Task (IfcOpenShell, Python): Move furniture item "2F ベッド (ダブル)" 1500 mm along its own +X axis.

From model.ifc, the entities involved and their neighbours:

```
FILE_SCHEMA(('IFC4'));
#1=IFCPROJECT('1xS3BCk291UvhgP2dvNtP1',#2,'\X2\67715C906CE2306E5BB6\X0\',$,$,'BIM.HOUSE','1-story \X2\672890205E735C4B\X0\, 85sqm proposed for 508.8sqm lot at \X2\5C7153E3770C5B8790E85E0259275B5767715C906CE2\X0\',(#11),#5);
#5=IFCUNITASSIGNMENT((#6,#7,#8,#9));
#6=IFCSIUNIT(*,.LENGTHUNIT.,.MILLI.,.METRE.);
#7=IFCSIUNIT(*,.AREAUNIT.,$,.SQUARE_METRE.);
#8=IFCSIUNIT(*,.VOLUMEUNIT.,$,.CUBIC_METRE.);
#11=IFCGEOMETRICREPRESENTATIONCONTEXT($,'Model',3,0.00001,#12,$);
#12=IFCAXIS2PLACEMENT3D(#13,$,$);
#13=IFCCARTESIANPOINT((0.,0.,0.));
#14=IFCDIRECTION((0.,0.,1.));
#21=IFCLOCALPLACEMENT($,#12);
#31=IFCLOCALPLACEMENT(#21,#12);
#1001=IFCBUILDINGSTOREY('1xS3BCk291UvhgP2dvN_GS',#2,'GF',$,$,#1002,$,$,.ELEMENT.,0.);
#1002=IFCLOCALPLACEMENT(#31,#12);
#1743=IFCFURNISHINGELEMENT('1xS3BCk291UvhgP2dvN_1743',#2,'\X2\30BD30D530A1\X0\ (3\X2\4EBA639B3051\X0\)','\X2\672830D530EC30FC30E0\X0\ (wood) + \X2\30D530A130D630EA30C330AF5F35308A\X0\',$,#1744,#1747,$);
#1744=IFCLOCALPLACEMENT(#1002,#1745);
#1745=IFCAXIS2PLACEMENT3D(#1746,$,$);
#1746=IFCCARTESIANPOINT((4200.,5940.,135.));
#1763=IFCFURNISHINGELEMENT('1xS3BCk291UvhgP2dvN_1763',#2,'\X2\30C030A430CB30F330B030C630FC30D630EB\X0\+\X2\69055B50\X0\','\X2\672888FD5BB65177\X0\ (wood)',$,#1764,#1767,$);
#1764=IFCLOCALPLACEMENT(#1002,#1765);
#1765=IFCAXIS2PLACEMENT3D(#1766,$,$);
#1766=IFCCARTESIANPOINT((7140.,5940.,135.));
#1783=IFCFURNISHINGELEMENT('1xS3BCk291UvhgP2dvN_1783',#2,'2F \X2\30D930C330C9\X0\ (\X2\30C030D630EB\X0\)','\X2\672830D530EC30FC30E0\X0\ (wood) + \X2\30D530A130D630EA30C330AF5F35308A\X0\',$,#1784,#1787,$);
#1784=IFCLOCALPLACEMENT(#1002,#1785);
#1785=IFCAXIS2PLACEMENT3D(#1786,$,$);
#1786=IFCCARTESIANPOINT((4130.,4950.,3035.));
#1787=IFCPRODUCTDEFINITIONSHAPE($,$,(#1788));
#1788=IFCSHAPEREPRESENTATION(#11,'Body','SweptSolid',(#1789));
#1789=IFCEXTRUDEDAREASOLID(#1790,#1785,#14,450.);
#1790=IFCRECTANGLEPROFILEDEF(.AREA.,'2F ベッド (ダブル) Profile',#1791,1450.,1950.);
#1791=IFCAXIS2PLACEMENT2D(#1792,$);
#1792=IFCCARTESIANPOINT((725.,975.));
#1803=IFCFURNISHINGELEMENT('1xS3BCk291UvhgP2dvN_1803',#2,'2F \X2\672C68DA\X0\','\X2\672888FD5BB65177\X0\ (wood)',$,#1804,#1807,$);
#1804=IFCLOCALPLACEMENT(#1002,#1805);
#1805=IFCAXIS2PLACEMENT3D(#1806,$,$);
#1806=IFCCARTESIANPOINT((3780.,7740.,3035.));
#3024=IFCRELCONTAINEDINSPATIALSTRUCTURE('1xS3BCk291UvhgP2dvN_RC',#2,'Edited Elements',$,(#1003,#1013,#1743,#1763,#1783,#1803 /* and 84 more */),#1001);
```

```python
import ifcopenshell
import ifcopenshell.api.geometry
import ifcopenshell.util.placement

model = ifcopenshell.open("model.ifc")

item = model.by_guid("1xS3BCk291UvhgP2dvN_1783")
matrix = ifcopenshell.util.placement.get_local_placement(item.ObjectPlacement)
matrix[:3, 3] += matrix[:3, 0] * 1500.0
ifcopenshell.api.geometry.edit_object_placement(model, product=item, matrix=matrix, is_si=False)

print(ifcopenshell.util.placement.get_local_placement(item.ObjectPlacement).round(3) + 0.0)

model.write("model-out.ifc")
```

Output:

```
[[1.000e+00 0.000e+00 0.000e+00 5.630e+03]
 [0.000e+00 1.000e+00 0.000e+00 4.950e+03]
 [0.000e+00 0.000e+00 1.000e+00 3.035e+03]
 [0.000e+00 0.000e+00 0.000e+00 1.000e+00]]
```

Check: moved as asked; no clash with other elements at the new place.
